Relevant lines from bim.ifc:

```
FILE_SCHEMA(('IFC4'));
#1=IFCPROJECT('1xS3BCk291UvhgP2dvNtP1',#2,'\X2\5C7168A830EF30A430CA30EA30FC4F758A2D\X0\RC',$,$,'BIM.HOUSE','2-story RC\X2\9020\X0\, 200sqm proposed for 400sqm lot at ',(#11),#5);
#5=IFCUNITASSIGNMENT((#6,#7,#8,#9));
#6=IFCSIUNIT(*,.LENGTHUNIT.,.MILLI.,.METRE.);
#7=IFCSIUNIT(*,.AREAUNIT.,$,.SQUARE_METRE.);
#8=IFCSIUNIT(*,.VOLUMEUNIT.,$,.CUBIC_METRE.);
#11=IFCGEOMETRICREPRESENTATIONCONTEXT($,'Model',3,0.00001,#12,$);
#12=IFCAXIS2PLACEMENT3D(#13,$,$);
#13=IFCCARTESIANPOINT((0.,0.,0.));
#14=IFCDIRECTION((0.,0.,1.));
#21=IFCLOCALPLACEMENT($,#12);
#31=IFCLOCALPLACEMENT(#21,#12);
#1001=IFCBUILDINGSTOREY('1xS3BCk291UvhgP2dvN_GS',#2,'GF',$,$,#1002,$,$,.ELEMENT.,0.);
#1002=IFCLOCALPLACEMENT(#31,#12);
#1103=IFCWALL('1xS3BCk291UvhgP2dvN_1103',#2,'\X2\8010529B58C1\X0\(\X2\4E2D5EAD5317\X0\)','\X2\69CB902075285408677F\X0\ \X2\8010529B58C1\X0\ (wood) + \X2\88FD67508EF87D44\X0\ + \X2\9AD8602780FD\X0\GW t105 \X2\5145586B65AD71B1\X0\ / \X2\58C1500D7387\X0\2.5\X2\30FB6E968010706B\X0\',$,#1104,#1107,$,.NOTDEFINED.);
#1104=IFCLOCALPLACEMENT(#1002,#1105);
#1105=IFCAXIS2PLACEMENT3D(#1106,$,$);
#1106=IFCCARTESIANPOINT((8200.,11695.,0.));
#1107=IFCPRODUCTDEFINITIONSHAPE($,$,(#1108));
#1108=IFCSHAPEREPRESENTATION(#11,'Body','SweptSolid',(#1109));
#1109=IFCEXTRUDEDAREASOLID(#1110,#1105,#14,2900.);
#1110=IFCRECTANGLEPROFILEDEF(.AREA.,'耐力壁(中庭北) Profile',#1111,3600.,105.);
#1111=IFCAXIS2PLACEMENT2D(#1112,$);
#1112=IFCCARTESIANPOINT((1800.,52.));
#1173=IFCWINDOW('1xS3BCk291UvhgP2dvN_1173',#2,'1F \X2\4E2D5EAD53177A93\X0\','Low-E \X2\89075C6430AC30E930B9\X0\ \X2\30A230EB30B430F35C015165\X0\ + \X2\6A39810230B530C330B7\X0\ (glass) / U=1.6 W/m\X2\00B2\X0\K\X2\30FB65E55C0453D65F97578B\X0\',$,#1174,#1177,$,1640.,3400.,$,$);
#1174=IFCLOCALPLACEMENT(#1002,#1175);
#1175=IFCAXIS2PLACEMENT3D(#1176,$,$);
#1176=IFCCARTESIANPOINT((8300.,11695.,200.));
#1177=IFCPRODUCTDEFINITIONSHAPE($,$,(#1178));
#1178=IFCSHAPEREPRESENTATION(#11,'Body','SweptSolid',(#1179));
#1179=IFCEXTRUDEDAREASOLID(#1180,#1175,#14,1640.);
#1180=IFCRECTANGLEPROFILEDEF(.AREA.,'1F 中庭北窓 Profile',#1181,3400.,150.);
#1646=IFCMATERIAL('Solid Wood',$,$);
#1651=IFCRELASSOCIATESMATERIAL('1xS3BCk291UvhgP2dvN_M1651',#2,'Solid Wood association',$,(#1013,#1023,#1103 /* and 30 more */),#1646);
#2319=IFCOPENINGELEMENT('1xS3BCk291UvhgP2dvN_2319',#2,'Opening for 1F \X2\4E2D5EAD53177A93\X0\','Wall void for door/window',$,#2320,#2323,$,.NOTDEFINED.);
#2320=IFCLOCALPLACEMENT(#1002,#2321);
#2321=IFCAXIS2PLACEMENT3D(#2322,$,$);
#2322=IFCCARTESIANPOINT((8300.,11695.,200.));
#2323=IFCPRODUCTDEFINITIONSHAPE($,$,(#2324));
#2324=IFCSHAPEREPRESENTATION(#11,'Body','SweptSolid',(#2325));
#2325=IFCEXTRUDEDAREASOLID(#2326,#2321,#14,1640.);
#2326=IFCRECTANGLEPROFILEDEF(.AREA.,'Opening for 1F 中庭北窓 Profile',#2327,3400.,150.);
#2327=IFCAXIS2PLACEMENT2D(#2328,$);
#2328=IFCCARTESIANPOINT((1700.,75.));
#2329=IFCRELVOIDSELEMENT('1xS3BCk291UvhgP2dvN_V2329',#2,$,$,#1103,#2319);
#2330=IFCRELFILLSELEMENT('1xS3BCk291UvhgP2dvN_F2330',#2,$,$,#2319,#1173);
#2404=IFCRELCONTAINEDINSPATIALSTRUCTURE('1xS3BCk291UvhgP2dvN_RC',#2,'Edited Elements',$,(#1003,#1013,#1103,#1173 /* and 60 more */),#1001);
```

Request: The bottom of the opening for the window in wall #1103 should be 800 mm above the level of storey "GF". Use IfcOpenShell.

```python
import numpy as np
import ifcopenshell
import ifcopenshell.api.geometry
import ifcopenshell.geom
import ifcopenshell.util.element
import ifcopenshell.util.placement
import ifcopenshell.util.shape
import ifcopenshell.util.unit

model = ifcopenshell.open("bim.ifc")
unit_scale = ifcopenshell.util.unit.calculate_unit_scale(model)

window = model.by_guid("1xS3BCk291UvhgP2dvN_1173")
opening = window.FillsVoids[0].RelatingOpeningElement
storey = ifcopenshell.util.element.get_container(window, ifc_class="IfcBuildingStorey")
level = ifcopenshell.util.placement.get_local_placement(storey.ObjectPlacement)[2, 3]

# The opening's origin need not be at the sill, so measure its lowest point.
shape = ifcopenshell.geom.create_shape(ifcopenshell.geom.settings(), opening)
bottom = ifcopenshell.util.shape.get_shape_bottom_elevation(shape, shape.geometry) / unit_scale
dz = level + 0.8 / unit_scale - bottom

shift = np.array([0.0, 0.0, dz])
# The window is not placed relative to its opening, so move both.
for product in (opening, window):
    matrix = ifcopenshell.util.placement.get_local_placement(product.ObjectPlacement)
    matrix[:3, 3] += shift
    ifcopenshell.api.geometry.edit_object_placement(model, product=product, matrix=matrix, is_si=False)

print(f"moved by {dz * unit_scale:+.3f} m")

model.write("bim_rev.ifc")
```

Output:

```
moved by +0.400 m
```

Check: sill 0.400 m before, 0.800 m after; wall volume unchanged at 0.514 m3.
